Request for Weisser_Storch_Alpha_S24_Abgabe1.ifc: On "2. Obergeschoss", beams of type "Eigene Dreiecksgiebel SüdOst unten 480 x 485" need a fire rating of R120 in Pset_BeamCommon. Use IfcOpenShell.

First a look at what the model holds.

```python
import ifcopenshell
import ifcopenshell.util.element

model = ifcopenshell.open("Weisser_Storch_Alpha_S24_Abgabe1.ifc")
print(model.schema)
storey = next(s for s in model.by_type("IfcBuildingStorey") if s.Name == "2. Obergeschoss")
beams = [e for e in ifcopenshell.util.element.get_decomposition(storey) if e.is_a("IfcBeam")]
seen = {}
for e in beams:
    element_type = ifcopenshell.util.element.get_type(e)
    key = (element_type.Name if element_type != e and element_type else None, ifcopenshell.util.element.get_pset(e, "Pset_BeamCommon", "FireRating"))
    seen[key] = seen.get(key, 0) + 1
for (name, value), count in sorted(seen.items(), key=str):
    print(count, "x", name, "|", value)
```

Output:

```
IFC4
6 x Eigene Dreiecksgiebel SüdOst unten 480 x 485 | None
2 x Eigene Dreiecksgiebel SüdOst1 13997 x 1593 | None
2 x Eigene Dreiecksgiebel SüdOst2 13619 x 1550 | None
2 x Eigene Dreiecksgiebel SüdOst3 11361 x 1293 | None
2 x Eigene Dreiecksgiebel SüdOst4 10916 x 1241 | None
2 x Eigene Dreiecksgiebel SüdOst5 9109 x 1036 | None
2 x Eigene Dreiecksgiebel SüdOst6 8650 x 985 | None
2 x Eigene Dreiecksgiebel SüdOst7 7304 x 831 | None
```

```python
import ifcopenshell
import ifcopenshell.api.pset
import ifcopenshell.util.element

model = ifcopenshell.open("Weisser_Storch_Alpha_S24_Abgabe1.ifc")

storey = next(s for s in model.by_type("IfcBuildingStorey") if s.Name == "2. Obergeschoss")
beams = [e for e in ifcopenshell.util.element.get_decomposition(storey) if e.is_a("IfcBeam")]

count = 0
for e in beams:
    element_type = ifcopenshell.util.element.get_type(e)
    if element_type in (None, e) or element_type.Name != "Eigene Dreiecksgiebel SüdOst unten 480 x 485":
        continue
    # add_pset returns the element's existing set when there is one.
    pset = ifcopenshell.api.pset.add_pset(model, product=e, name="Pset_BeamCommon")
    ifcopenshell.api.pset.edit_pset(model, pset=pset, properties={"FireRating": "R120"})
    count += 1

print(count, "beams updated")

model.write("Weisser_Storch_Alpha_S24_Abgabe1_updated.ifc")
```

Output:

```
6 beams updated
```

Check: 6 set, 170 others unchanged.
